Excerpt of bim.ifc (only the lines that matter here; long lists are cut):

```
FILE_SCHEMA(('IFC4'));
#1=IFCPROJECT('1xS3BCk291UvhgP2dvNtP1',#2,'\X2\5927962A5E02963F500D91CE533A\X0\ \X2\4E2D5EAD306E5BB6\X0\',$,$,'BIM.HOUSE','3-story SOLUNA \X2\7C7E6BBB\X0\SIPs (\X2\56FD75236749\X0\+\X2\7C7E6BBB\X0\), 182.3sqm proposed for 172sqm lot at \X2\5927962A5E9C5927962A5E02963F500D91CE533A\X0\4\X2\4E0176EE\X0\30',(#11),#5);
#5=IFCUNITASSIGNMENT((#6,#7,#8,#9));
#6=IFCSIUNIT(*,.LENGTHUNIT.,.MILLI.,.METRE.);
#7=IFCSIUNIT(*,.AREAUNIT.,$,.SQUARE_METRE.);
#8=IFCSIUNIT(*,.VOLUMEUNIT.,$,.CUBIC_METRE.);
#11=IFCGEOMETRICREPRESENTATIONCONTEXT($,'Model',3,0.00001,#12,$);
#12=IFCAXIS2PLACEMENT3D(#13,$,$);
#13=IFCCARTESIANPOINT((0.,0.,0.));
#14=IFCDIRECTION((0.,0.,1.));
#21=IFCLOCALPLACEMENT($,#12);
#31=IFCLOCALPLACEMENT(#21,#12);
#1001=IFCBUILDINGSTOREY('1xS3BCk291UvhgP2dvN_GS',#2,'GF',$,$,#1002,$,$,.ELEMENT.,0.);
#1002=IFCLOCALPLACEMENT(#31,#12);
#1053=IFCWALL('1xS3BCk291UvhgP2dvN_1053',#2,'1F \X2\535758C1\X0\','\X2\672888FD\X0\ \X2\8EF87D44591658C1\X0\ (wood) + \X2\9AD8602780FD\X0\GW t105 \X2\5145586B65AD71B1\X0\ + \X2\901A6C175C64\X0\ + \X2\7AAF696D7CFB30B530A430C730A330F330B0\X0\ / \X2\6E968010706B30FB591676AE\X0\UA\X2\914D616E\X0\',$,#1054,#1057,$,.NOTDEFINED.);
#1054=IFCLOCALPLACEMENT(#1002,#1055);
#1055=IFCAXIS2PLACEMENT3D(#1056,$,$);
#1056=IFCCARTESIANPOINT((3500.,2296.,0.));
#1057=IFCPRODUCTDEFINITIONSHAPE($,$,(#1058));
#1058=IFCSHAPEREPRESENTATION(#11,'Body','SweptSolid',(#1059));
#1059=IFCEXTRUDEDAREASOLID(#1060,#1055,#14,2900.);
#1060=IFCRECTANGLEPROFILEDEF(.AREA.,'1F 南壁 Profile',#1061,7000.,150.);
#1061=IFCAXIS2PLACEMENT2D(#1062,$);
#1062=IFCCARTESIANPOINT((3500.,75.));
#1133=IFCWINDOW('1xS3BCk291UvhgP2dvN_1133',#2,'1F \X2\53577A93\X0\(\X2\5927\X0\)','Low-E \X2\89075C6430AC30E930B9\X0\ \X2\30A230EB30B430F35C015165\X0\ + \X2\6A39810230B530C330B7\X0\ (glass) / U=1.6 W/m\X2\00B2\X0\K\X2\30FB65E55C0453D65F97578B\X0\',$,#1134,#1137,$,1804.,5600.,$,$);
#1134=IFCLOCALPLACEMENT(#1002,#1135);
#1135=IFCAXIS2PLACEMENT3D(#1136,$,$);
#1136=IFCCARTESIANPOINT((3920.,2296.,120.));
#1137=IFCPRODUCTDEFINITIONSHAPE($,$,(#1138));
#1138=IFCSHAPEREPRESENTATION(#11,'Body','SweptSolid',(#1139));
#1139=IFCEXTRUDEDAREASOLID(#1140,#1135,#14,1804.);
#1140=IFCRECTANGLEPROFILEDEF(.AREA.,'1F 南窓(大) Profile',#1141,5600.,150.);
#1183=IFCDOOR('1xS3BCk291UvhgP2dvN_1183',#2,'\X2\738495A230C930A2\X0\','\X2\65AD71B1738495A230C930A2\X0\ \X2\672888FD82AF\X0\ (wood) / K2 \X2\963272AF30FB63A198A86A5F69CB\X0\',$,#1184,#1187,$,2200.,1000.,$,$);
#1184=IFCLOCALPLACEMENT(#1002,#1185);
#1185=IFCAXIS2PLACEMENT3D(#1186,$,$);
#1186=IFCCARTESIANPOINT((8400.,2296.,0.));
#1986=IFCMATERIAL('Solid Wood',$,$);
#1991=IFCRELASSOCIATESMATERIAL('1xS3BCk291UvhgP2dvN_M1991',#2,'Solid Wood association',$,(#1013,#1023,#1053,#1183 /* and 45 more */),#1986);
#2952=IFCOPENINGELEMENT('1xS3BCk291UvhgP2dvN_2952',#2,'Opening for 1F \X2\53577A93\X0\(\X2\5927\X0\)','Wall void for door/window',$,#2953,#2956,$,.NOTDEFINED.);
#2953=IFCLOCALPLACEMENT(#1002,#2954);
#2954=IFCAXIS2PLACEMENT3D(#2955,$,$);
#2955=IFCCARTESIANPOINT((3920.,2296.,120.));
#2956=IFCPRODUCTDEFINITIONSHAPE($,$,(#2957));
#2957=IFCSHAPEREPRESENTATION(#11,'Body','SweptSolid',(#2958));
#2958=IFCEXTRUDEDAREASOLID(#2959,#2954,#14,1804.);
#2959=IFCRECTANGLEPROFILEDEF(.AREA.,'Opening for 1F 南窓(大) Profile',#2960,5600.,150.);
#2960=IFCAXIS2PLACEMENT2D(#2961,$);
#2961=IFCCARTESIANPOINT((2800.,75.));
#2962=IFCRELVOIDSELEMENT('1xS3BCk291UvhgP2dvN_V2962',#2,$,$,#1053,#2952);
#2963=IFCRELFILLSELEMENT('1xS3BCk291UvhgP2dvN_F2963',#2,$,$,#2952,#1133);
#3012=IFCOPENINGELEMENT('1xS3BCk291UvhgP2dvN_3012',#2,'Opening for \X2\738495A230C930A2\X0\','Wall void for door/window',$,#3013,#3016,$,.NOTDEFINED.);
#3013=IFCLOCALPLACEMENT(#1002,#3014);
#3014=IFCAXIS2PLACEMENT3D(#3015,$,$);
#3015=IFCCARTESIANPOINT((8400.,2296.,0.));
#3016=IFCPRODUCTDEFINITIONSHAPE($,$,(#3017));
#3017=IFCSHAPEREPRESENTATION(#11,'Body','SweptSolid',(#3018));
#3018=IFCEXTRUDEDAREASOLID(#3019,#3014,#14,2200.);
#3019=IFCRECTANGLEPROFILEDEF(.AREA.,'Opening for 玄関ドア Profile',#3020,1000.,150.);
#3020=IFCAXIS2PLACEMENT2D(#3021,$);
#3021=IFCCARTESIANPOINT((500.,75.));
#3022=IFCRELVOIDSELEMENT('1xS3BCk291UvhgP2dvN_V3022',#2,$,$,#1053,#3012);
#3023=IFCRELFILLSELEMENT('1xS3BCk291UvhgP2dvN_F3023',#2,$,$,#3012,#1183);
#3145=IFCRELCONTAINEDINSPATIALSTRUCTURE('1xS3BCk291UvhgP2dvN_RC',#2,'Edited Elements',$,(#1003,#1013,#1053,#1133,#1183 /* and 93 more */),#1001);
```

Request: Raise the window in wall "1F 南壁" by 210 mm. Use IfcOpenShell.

```python
import numpy as np
import ifcopenshell
import ifcopenshell.api.geometry
import ifcopenshell.util.placement
import ifcopenshell.util.unit

model = ifcopenshell.open("bim.ifc")
unit_scale = ifcopenshell.util.unit.calculate_unit_scale(model)

window = model.by_id(1133)
opening = window.FillsVoids[0].RelatingOpeningElement
dz = 210.0

shift = np.array([0.0, 0.0, dz])
# The window is not placed relative to its opening, so move both.
for product in (opening, window):
    matrix = ifcopenshell.util.placement.get_local_placement(product.ObjectPlacement)
    matrix[:3, 3] += shift
    ifcopenshell.api.geometry.edit_object_placement(model, product=product, matrix=matrix, is_si=False)

print(f"moved by {dz * unit_scale:+.3f} m")

model.write("bim_rev.ifc")
```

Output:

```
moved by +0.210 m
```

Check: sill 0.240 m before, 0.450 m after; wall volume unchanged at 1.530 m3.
